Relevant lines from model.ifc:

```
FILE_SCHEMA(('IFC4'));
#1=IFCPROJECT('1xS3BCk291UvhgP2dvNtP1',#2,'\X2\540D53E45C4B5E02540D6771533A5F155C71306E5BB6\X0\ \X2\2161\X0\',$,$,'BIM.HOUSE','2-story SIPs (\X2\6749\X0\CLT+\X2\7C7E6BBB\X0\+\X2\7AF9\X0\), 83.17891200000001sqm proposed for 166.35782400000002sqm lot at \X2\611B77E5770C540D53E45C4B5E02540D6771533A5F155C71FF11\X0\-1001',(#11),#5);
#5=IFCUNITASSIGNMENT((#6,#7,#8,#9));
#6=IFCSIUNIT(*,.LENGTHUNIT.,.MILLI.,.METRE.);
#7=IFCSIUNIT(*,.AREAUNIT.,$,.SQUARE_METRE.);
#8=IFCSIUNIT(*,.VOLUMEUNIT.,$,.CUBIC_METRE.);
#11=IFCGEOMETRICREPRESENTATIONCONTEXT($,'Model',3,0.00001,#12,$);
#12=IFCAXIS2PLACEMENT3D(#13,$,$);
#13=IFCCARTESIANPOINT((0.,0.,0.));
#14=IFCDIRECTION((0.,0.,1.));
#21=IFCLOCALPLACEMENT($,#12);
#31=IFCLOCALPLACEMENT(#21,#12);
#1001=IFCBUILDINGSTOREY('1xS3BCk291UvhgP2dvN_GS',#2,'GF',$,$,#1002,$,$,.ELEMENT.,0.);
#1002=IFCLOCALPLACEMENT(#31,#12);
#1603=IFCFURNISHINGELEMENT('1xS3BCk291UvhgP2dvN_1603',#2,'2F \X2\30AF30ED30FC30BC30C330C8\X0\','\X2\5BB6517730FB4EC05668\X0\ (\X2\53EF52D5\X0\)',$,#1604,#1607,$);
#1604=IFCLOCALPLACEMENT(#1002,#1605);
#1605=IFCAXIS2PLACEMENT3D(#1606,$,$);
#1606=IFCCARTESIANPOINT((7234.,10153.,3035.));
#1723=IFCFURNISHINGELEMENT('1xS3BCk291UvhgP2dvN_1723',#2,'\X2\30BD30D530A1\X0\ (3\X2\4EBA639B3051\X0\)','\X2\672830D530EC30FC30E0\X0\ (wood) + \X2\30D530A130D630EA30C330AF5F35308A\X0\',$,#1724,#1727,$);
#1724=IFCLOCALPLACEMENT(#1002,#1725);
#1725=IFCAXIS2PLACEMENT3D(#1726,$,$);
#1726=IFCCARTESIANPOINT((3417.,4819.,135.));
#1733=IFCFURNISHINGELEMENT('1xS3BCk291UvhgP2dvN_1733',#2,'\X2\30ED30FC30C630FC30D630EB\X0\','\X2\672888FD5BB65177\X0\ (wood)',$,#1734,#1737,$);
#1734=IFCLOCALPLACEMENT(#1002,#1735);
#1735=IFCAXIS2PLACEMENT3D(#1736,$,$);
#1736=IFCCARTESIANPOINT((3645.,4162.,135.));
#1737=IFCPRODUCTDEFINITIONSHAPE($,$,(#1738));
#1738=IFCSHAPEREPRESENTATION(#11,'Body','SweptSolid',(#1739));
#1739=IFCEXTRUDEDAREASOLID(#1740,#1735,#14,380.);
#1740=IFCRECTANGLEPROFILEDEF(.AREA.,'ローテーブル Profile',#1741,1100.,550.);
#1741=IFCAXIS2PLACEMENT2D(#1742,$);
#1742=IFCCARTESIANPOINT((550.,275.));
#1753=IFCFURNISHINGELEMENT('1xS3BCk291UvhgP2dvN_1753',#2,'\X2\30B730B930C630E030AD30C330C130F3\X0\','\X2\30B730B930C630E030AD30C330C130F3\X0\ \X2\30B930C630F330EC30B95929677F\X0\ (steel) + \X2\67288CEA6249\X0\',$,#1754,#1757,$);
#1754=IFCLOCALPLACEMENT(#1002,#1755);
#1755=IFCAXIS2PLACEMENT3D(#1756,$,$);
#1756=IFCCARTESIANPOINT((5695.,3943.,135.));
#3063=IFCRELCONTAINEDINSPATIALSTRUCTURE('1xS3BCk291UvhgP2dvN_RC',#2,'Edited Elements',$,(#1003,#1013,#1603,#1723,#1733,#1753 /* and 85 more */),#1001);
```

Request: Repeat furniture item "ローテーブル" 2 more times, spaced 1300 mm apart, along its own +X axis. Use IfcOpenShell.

```python
import ifcopenshell
import ifcopenshell.api.geometry
import ifcopenshell.api.root
import ifcopenshell.util.element
import ifcopenshell.util.placement
import ifcopenshell.util.unit

model = ifcopenshell.open("model.ifc")
unit_scale = ifcopenshell.util.unit.calculate_unit_scale(model)


def reuse_history(source, copy):
    """copy_class also copies each property set's owner history, people and application; keep the originals."""
    for rel in copy.IsDefinedBy:
        if rel.is_a("IfcRelDefinesByProperties") and (history := rel.RelatingPropertyDefinition.OwnerHistory):
            rel.RelatingPropertyDefinition.OwnerHistory = source.OwnerHistory
            ifcopenshell.util.element.remove_deep2(model, history)


source = model.by_guid("1xS3BCk291UvhgP2dvN_1733")
base = ifcopenshell.util.placement.get_local_placement(source.ObjectPlacement)
step = base[:3, 0] * 1.3 / unit_scale

for i in range(1, 3):
    copy = ifcopenshell.api.root.copy_class(model, product=source)
    copy.Representation = ifcopenshell.util.element.copy_deep(
        model, source.Representation, exclude=["IfcGeometricRepresentationContext", "IfcRepresentationMap"]
    )
    reuse_history(source, copy)
    matrix = base.copy()
    matrix[:3, 3] += i * step
    print("added at", matrix[:3, 3].round(3) + 0.0)
    ifcopenshell.api.geometry.edit_object_placement(model, product=copy, matrix=matrix, is_si=False)

model.write("model-out.ifc")
```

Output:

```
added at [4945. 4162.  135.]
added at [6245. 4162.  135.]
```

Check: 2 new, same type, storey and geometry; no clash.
